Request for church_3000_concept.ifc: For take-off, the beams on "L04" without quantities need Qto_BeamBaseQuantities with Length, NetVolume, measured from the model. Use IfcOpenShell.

First a look at what the model holds.

```python
import ifcopenshell
import ifcopenshell.util.element
import ifcopenshell.util.unit

model = ifcopenshell.open("church_3000_concept.ifc")
print(model.schema)
for unit_type in ("LENGTHUNIT", "AREAUNIT", "VOLUMEUNIT"):
    print(unit_type, ifcopenshell.util.unit.calculate_unit_scale(model, unit_type))
storey = next(s for s in model.by_type("IfcBuildingStorey") if s.Name == "L04")
beams = [e for e in ifcopenshell.util.element.get_decomposition(storey) if e.is_a("IfcBeam")]
for e in sorted(beams, key=lambda e: e.id()):
    print(e.id(), e.is_a(), e.Name, list(ifcopenshell.util.element.get_psets(e, qtos_only=True)), sep=" | ")
```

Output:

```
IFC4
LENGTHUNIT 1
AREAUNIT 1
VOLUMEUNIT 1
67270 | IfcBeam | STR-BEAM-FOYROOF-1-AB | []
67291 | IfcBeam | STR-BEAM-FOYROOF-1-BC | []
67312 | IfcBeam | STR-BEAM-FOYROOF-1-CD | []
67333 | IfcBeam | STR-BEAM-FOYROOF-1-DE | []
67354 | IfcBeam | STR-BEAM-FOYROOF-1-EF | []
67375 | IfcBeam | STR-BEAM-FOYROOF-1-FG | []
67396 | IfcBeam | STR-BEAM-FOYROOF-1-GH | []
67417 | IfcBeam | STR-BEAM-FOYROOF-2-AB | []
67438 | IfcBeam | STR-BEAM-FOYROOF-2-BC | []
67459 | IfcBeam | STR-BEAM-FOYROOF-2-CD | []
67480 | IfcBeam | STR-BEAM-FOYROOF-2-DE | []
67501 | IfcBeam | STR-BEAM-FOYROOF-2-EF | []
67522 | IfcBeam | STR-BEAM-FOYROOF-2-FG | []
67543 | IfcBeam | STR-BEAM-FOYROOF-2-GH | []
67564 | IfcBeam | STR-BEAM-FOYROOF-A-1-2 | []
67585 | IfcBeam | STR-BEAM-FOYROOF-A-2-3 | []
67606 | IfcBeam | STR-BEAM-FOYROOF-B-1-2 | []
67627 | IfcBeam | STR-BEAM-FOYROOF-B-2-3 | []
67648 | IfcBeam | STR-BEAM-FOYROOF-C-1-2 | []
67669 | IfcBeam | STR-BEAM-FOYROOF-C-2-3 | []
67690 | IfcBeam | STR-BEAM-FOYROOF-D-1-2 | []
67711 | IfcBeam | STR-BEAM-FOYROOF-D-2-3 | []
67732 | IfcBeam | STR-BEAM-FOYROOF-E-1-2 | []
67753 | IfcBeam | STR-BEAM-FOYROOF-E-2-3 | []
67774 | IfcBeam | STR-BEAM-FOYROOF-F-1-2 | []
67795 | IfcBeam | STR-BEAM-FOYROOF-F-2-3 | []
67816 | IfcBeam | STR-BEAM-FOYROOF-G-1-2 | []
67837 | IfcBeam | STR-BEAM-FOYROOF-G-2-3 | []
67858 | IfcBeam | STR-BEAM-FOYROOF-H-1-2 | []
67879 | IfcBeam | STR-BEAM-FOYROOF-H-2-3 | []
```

```python
import ifcopenshell
import ifcopenshell.api.pset
import ifcopenshell.geom
import ifcopenshell.util.element
import ifcopenshell.util.shape
import ifcopenshell.util.unit

model = ifcopenshell.open("church_3000_concept.ifc")
unit_scale = ifcopenshell.util.unit.calculate_unit_scale(model)
volume_scale = ifcopenshell.util.unit.calculate_unit_scale(model, "VOLUMEUNIT")
settings = ifcopenshell.geom.settings()

storey = next(s for s in model.by_type("IfcBuildingStorey") if s.Name == "L04")
beams = [e for e in ifcopenshell.util.element.get_decomposition(storey) if e.is_a("IfcBeam")]

for e in sorted(beams, key=lambda e: e.id()):
    if ifcopenshell.util.element.get_psets(e, qtos_only=True, should_inherit=False):
        continue
    # Geometry comes back in metres, in the element's own axes.
    shape = ifcopenshell.geom.create_shape(settings, e)
    values = {
        "Length": ifcopenshell.util.shape.get_max_xyz(shape.geometry) / unit_scale,
        "NetVolume": ifcopenshell.util.shape.get_volume(shape.geometry) / volume_scale,
    }
    qto = ifcopenshell.api.pset.add_qto(model, product=e, name="Qto_BeamBaseQuantities")
    ifcopenshell.api.pset.edit_qto(model, qto=qto, properties=values)
    print(e.id(), {k: round(v, 3) for k, v in values.items()})

model.write("church_3000_concept-out.ifc")
```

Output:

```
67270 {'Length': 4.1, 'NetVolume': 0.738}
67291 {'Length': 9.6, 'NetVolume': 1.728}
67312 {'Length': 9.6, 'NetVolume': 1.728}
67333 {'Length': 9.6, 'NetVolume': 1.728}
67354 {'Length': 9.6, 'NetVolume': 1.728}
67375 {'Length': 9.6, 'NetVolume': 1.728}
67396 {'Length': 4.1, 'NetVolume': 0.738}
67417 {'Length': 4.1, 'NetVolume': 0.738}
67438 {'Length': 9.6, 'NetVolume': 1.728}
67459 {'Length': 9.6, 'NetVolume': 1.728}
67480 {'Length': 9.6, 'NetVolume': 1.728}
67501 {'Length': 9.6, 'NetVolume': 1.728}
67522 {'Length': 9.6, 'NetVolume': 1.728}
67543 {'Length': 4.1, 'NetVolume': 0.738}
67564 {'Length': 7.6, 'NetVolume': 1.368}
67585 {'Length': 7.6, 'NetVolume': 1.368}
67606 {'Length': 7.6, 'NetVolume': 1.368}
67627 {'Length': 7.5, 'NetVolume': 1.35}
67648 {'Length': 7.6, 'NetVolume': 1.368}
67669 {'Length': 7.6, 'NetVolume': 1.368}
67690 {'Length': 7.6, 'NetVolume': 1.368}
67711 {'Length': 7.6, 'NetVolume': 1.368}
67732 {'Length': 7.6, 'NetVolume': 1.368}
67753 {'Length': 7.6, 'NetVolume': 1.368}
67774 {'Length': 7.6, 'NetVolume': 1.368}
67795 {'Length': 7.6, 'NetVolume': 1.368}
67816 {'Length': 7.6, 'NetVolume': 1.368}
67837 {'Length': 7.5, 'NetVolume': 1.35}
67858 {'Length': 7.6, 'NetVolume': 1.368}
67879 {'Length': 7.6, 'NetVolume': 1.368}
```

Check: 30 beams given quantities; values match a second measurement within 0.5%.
